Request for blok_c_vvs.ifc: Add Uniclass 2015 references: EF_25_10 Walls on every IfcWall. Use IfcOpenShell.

First a look at what the model holds.

```python
import ifcopenshell

model = ifcopenshell.open("blok_c_vvs.ifc")
print(model.schema)
print("classifications:", [c.Name for c in model.by_type("IfcClassification")])
for ifc_class in ("IfcDoor", "IfcRoof", "IfcStair", "IfcWall", "IfcWindow"):
    print(ifc_class, len(model.by_type(ifc_class)))
```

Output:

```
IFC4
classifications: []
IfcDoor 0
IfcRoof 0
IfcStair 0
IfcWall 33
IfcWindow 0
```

```python
import ifcopenshell
import ifcopenshell.api.classification

model = ifcopenshell.open("blok_c_vvs.ifc")

system = ifcopenshell.api.classification.add_classification(model, classification="Uniclass 2015")

codes = {
    "IfcWall": ("EF_25_10", "Walls"),
}
for ifc_class, (code, name) in codes.items():
    products = model.by_type(ifc_class)
    ifcopenshell.api.classification.add_reference(
        model, products=products, classification=system, identification=code, name=name
    )
    print(code, len(products))

model.write("blok_c_vvs_updated.ifc")
```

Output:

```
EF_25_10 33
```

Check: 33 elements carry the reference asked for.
